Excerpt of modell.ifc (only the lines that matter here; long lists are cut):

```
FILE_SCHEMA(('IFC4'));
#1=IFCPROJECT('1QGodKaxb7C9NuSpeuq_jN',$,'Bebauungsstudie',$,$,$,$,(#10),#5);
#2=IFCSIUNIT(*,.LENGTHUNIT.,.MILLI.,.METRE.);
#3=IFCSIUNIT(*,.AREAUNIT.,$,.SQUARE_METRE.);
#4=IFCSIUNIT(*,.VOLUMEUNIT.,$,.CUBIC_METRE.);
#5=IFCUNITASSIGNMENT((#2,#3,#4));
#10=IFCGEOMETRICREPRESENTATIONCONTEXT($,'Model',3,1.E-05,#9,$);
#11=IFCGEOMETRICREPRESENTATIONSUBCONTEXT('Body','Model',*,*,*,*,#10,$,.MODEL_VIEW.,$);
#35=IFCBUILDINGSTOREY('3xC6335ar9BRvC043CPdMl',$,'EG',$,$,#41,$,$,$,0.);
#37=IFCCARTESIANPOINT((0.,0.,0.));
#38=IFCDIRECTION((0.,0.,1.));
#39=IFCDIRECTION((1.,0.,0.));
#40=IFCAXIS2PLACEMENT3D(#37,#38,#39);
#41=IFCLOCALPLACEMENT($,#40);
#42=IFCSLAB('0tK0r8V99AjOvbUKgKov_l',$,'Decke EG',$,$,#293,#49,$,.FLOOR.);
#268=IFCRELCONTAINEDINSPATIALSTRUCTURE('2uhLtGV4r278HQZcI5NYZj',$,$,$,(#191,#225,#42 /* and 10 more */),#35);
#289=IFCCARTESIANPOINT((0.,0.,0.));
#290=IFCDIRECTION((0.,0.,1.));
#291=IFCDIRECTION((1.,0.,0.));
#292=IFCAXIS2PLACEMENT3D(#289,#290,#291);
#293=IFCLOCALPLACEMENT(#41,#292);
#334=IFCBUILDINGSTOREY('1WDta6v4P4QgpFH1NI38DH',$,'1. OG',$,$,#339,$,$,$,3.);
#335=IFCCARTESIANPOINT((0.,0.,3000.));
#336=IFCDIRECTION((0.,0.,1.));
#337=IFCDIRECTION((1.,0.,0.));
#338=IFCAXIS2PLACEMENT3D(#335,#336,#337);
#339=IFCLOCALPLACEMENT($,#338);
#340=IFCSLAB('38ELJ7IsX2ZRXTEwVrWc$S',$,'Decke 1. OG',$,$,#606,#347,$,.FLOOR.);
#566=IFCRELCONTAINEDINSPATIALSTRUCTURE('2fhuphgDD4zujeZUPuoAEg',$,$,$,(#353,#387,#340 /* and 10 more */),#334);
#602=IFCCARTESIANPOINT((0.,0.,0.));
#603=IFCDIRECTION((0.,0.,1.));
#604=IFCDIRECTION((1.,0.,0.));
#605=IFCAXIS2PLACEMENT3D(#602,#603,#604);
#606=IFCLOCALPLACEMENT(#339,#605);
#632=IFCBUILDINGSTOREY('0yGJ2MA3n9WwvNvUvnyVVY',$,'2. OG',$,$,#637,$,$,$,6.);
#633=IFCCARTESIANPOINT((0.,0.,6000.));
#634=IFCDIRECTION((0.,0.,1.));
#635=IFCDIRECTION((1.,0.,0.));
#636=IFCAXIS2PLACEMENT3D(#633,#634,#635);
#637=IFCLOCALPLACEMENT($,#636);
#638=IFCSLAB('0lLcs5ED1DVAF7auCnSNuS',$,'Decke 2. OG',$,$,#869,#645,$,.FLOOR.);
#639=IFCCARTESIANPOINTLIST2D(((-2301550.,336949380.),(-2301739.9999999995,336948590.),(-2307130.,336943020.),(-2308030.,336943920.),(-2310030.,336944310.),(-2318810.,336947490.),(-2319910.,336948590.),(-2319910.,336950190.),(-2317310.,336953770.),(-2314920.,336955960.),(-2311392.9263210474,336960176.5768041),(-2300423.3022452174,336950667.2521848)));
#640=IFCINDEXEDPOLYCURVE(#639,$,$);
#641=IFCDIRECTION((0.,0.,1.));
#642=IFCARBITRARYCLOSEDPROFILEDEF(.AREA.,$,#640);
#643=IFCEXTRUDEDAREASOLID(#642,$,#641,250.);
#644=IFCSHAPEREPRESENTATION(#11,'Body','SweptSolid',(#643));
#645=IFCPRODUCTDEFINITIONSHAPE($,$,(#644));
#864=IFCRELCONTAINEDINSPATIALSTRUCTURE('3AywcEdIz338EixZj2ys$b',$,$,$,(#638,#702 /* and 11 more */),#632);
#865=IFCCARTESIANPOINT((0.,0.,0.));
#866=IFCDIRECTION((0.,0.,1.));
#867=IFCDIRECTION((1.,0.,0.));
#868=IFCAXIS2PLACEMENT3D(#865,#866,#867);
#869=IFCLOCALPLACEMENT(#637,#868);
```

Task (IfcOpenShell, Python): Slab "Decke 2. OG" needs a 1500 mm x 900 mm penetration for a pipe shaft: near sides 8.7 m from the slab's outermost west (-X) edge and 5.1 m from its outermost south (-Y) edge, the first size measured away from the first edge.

```python
import numpy as np
import ifcopenshell
import ifcopenshell.api.feature
import ifcopenshell.api.geometry
import ifcopenshell.api.root
import ifcopenshell.geom
import ifcopenshell.util.placement
import ifcopenshell.util.representation
import ifcopenshell.util.shape
import ifcopenshell.util.unit

model = ifcopenshell.open("modell.ifc")
unit_scale = ifcopenshell.util.unit.calculate_unit_scale(model)
settings = ifcopenshell.geom.settings()


def volume(element):
    """Net volume in cubic metres, openings subtracted."""
    shape = ifcopenshell.geom.create_shape(settings, element)
    return ifcopenshell.util.shape.get_volume(shape.geometry)


slab = model.by_id(638)
before = volume(slab)

# Extent in the slab's own axes, in metres. The edges named are its -X and -Y sides.
slab_shape = ifcopenshell.geom.create_shape(settings, slab)
vertices = ifcopenshell.util.shape.get_vertices(slab_shape.geometry)
x_min, y_min, bottom = vertices.min(axis=0)
top = vertices[:, 2].max()

opening = ifcopenshell.api.root.create_entity(model, ifc_class="IfcOpeningElement", name="Pipe shaft opening", predefined_type="OPENING")
context = ifcopenshell.util.representation.get_context(model, "Model", "Body", "MODEL_VIEW")
width, depth = 1.5, 0.9
outline = [(0.0, 0.0), (width, 0.0), (width, depth), (0.0, depth), (0.0, 0.0)]
# Overshoot both faces by 50 mm so the cut is clean.
shape = ifcopenshell.api.geometry.add_slab_representation(
    model, context=context, depth=top - bottom + 0.1, polyline=outline
)
ifcopenshell.api.geometry.assign_representation(model, product=opening, representation=shape)

matrix = ifcopenshell.util.placement.get_local_placement(slab.ObjectPlacement)
matrix[:, 3] = matrix @ np.append(np.array([x_min + 8.7, y_min + 5.1, bottom - 0.05]) / unit_scale, 1.0)
ifcopenshell.api.geometry.edit_object_placement(model, product=opening, matrix=matrix, is_si=False)
ifcopenshell.api.feature.add_feature(model, feature=opening, element=slab)

after = volume(slab)

print(f"slab volume {before:.3f} -> {after:.3f} m3")

model.write("modell_v2.ifc")
```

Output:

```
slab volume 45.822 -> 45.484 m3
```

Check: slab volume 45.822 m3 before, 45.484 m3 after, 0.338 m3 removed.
